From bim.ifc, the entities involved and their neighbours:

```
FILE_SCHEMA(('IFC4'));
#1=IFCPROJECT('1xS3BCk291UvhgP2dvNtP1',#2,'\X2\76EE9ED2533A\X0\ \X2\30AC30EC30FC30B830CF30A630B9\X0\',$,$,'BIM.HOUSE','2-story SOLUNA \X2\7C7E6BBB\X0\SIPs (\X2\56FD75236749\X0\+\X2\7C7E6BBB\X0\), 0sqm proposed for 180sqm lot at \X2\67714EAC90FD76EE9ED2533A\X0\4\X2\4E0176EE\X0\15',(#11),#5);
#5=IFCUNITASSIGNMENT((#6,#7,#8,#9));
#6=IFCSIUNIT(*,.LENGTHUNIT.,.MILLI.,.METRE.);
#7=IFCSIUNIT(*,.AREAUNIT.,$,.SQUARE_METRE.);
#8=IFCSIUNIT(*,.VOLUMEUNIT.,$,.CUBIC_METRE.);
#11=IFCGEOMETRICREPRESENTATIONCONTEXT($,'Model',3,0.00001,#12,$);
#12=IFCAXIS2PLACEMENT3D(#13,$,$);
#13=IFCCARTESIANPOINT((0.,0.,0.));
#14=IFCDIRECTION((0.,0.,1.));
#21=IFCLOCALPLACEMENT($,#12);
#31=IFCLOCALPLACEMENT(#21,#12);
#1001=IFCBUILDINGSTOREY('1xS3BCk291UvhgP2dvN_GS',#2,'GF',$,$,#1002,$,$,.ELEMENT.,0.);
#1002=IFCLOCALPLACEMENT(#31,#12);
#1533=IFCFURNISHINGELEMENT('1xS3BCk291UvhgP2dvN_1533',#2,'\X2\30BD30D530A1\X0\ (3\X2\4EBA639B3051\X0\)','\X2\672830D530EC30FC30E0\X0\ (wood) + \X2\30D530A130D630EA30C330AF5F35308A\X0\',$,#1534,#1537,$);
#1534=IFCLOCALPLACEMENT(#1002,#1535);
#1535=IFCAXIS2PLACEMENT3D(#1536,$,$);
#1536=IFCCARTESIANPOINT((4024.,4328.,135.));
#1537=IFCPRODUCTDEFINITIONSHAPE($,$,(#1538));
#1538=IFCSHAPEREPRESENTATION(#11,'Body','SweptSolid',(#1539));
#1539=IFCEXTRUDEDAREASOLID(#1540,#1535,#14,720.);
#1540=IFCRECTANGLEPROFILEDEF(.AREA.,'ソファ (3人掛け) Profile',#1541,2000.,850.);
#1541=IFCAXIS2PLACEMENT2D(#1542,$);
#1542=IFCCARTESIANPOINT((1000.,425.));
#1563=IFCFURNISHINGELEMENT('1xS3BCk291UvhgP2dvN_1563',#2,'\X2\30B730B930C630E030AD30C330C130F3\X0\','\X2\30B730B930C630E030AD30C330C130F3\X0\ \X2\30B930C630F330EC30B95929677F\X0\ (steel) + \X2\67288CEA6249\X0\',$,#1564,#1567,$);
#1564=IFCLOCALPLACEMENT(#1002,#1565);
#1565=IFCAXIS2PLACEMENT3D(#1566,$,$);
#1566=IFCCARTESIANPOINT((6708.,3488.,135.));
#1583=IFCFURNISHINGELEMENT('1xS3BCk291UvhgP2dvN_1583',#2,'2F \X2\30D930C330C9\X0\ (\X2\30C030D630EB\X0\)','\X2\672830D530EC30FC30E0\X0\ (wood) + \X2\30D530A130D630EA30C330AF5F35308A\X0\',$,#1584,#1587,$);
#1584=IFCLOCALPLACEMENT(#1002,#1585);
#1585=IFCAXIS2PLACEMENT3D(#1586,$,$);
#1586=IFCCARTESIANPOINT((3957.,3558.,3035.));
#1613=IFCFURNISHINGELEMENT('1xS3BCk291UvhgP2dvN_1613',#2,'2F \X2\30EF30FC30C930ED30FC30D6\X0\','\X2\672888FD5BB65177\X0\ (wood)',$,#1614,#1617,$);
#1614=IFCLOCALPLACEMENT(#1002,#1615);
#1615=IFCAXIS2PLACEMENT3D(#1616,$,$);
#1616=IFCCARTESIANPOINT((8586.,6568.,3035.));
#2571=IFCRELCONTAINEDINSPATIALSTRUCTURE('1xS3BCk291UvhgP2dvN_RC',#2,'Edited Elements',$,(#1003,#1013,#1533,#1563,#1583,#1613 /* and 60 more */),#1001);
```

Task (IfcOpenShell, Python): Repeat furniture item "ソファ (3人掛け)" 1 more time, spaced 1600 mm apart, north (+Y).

```python
import numpy as np
import ifcopenshell
import ifcopenshell.api.geometry
import ifcopenshell.api.root
import ifcopenshell.util.element
import ifcopenshell.util.placement

model = ifcopenshell.open("bim.ifc")


def reuse_history(source, copy):
    """copy_class also copies each property set's owner history, people and application; keep the originals."""
    for rel in copy.IsDefinedBy:
        if rel.is_a("IfcRelDefinesByProperties") and (history := rel.RelatingPropertyDefinition.OwnerHistory):
            rel.RelatingPropertyDefinition.OwnerHistory = source.OwnerHistory
            ifcopenshell.util.element.remove_deep2(model, history)


source = model.by_guid("1xS3BCk291UvhgP2dvN_1533")
base = ifcopenshell.util.placement.get_local_placement(source.ObjectPlacement)
step = np.array([0.0, 1.0, 0.0]) * 1600.0

for i in range(1, 2):
    copy = ifcopenshell.api.root.copy_class(model, product=source)
    copy.Representation = ifcopenshell.util.element.copy_deep(
        model, source.Representation, exclude=["IfcGeometricRepresentationContext", "IfcRepresentationMap"]
    )
    reuse_history(source, copy)
    matrix = base.copy()
    matrix[:3, 3] += i * step
    print("added at", matrix[:3, 3].round(3) + 0.0)
    ifcopenshell.api.geometry.edit_object_placement(model, product=copy, matrix=matrix, is_si=False)

model.write("bim_edited.ifc")
```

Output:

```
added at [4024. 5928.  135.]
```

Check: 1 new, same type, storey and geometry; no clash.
